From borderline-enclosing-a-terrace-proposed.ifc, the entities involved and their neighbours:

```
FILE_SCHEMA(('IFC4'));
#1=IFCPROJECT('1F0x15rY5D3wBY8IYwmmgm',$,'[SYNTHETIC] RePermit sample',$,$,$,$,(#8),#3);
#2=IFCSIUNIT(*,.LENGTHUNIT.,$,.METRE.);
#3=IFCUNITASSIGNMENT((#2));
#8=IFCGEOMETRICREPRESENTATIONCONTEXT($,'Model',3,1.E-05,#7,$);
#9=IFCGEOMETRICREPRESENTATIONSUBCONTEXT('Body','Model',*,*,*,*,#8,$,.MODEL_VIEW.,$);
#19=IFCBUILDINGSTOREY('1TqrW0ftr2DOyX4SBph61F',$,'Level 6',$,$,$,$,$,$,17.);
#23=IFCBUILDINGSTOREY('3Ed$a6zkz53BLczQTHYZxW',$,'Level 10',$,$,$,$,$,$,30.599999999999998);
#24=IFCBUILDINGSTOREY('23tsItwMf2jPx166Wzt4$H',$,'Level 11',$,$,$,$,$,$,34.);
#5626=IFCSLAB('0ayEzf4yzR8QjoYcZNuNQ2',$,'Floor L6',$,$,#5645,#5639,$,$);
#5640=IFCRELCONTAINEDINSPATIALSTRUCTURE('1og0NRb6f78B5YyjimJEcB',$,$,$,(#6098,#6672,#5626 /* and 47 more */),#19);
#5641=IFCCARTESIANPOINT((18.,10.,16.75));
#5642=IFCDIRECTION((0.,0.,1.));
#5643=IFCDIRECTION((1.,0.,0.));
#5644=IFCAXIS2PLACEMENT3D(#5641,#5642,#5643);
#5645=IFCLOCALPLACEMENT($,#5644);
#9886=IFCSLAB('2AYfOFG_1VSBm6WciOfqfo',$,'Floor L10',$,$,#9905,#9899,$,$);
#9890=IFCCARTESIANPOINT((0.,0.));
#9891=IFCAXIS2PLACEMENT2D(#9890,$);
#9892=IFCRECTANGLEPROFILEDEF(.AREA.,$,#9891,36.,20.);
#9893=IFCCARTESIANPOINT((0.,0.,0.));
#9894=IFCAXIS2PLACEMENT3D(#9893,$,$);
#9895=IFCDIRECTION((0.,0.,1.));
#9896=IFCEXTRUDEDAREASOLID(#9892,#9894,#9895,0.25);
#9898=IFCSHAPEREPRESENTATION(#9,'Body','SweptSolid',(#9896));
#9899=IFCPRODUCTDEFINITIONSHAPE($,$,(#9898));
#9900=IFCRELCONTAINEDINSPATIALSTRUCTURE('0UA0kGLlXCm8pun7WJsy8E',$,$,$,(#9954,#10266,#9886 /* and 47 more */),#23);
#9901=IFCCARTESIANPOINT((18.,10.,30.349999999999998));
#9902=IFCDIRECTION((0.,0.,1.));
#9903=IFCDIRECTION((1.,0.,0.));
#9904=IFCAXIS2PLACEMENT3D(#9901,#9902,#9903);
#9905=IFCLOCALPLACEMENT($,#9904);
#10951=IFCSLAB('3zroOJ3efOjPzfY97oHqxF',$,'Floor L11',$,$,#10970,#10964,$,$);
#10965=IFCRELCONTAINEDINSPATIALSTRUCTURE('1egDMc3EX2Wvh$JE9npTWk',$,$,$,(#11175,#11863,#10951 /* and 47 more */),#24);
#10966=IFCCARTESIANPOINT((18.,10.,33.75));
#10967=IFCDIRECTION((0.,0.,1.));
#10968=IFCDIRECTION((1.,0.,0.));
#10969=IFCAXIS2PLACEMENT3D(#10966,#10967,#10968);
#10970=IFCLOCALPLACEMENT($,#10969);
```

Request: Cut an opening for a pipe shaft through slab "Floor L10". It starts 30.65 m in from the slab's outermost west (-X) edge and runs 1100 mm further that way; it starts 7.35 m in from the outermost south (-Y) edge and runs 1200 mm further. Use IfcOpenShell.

```python
import numpy as np
import ifcopenshell
import ifcopenshell.api.feature
import ifcopenshell.api.geometry
import ifcopenshell.api.root
import ifcopenshell.geom
import ifcopenshell.util.placement
import ifcopenshell.util.representation
import ifcopenshell.util.shape
import ifcopenshell.util.unit

model = ifcopenshell.open("borderline-enclosing-a-terrace-proposed.ifc")
unit_scale = ifcopenshell.util.unit.calculate_unit_scale(model)
settings = ifcopenshell.geom.settings()


def volume(element):
    """Net volume in cubic metres, openings subtracted."""
    shape = ifcopenshell.geom.create_shape(settings, element)
    return ifcopenshell.util.shape.get_volume(shape.geometry)


slab = model.by_id(9886)
before = volume(slab)

# Extent in the slab's own axes, in metres. The edges named are its -X and -Y sides.
slab_shape = ifcopenshell.geom.create_shape(settings, slab)
vertices = ifcopenshell.util.shape.get_vertices(slab_shape.geometry)
x_min, y_min, bottom = vertices.min(axis=0)
top = vertices[:, 2].max()

opening = ifcopenshell.api.root.create_entity(model, ifc_class="IfcOpeningElement", name="Pipe shaft opening", predefined_type="OPENING")
context = ifcopenshell.util.representation.get_context(model, "Model", "Body", "MODEL_VIEW")
width, depth = 1.1, 1.2
outline = [(0.0, 0.0), (width, 0.0), (width, depth), (0.0, depth), (0.0, 0.0)]
# Overshoot both faces by 50 mm so the cut is clean.
shape = ifcopenshell.api.geometry.add_slab_representation(
    model, context=context, depth=top - bottom + 0.1, polyline=outline
)
ifcopenshell.api.geometry.assign_representation(model, product=opening, representation=shape)

matrix = ifcopenshell.util.placement.get_local_placement(slab.ObjectPlacement)
matrix[:, 3] = matrix @ np.append(np.array([x_min + 30.65, y_min + 7.35, bottom - 0.05]) / unit_scale, 1.0)
ifcopenshell.api.geometry.edit_object_placement(model, product=opening, matrix=matrix, is_si=False)
ifcopenshell.api.feature.add_feature(model, feature=opening, element=slab)

after = volume(slab)

print(f"slab volume {before:.3f} -> {after:.3f} m3")

model.write("borderline-enclosing-a-terrace-proposed_edited.ifc")
```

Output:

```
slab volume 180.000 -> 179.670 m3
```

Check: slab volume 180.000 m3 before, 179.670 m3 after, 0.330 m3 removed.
